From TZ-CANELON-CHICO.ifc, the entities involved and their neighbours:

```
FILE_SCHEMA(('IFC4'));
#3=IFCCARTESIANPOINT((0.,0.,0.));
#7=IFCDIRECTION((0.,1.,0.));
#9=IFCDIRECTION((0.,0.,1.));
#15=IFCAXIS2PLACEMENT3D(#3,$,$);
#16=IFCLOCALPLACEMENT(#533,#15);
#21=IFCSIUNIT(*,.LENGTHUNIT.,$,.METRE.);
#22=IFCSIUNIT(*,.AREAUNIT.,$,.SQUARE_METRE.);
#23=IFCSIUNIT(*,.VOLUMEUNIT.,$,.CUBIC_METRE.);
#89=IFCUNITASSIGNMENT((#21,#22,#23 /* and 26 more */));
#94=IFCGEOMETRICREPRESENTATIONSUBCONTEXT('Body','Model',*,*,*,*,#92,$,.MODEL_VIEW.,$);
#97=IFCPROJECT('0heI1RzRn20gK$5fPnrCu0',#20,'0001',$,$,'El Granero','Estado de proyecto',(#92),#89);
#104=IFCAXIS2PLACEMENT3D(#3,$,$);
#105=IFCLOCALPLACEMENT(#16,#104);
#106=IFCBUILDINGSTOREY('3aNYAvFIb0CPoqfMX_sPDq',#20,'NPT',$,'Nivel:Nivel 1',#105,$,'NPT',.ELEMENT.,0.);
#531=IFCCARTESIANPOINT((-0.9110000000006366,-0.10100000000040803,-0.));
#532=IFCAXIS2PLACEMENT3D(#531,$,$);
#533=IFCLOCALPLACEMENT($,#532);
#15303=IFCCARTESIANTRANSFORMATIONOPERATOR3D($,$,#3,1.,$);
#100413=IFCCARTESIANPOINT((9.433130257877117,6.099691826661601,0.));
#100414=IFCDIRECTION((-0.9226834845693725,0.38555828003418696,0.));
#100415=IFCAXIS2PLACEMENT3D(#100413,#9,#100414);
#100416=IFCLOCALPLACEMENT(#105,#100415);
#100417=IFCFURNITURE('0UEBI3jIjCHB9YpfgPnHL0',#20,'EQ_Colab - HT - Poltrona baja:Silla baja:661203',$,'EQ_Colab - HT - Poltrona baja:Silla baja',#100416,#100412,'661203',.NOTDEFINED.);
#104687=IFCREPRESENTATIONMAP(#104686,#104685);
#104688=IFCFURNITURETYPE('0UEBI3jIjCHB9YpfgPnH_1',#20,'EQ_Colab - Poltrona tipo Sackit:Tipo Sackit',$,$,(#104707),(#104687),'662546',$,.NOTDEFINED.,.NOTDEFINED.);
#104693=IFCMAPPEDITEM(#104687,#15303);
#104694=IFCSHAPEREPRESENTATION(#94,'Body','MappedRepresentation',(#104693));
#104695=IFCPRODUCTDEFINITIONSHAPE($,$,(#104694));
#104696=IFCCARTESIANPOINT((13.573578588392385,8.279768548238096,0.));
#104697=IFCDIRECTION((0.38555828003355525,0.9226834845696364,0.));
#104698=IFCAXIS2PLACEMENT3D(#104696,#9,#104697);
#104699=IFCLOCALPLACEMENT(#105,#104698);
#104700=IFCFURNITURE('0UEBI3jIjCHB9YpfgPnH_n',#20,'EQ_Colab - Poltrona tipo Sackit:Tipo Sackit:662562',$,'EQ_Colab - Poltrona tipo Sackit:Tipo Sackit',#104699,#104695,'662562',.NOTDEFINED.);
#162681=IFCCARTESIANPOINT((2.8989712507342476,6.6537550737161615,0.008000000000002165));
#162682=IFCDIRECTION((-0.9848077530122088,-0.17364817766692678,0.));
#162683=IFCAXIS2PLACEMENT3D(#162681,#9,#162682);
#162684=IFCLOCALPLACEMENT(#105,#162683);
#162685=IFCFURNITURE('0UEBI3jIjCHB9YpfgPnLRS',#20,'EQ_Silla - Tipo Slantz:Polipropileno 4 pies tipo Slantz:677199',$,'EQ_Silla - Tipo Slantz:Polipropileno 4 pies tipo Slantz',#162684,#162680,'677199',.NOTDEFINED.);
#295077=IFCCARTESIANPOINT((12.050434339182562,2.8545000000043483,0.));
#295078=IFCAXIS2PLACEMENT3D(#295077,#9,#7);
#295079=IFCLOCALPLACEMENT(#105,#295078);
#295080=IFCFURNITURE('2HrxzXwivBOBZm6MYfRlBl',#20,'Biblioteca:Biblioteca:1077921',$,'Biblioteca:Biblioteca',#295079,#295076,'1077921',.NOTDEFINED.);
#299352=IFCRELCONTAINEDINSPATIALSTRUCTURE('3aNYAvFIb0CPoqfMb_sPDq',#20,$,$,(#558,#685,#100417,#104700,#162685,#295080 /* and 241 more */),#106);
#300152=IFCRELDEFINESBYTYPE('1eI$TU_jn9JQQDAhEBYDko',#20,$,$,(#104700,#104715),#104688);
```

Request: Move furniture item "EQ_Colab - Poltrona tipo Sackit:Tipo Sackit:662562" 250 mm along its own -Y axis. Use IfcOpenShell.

```python
import ifcopenshell
import ifcopenshell.api.geometry
import ifcopenshell.util.placement

model = ifcopenshell.open("TZ-CANELON-CHICO.ifc")

item = model.by_guid("0UEBI3jIjCHB9YpfgPnH_n")
matrix = ifcopenshell.util.placement.get_local_placement(item.ObjectPlacement)
matrix[:3, 3] -= matrix[:3, 1] * 0.25
ifcopenshell.api.geometry.edit_object_placement(model, product=item, matrix=matrix, is_si=False)

print(ifcopenshell.util.placement.get_local_placement(item.ObjectPlacement).round(3) + 0.0)

model.write("TZ-CANELON-CHICO_updated.ifc")
```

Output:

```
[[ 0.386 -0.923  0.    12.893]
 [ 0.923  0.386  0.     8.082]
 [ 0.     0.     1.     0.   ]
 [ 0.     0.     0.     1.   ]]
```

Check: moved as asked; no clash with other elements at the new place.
